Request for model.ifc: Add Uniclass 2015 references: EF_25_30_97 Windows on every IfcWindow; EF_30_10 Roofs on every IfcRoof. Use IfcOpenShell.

First a look at what the model holds.

```python
import ifcopenshell

model = ifcopenshell.open("model.ifc")
print(model.schema)
print("classifications:", [c.Name for c in model.by_type("IfcClassification")])
for ifc_class in ("IfcDoor", "IfcRoof", "IfcStair", "IfcWall", "IfcWindow"):
    print(ifc_class, len(model.by_type(ifc_class)))
```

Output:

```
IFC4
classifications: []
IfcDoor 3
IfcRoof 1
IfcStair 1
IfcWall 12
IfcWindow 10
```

```python
import ifcopenshell
import ifcopenshell.api.classification

model = ifcopenshell.open("model.ifc")

system = ifcopenshell.api.classification.add_classification(model, classification="Uniclass 2015")

codes = {
    "IfcWindow": ("EF_25_30_97", "Windows"),
    "IfcRoof": ("EF_30_10", "Roofs"),
}
for ifc_class, (code, name) in codes.items():
    products = model.by_type(ifc_class)
    ifcopenshell.api.classification.add_reference(
        model, products=products, classification=system, identification=code, name=name
    )
    print(code, len(products))

model.write("model_updated.ifc")
```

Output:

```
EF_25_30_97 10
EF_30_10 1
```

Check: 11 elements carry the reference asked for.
